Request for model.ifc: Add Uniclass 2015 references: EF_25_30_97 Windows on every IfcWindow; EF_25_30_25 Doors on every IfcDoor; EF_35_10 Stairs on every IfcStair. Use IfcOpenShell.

First a look at what the model holds.

```python
import ifcopenshell

model = ifcopenshell.open("model.ifc")
print(model.schema)
print("classifications:", [c.Name for c in model.by_type("IfcClassification")])
for ifc_class in ("IfcDoor", "IfcRoof", "IfcStair", "IfcWall", "IfcWindow"):
    print(ifc_class, len(model.by_type(ifc_class)))
```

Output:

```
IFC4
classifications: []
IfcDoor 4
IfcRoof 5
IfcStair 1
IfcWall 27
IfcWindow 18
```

```python
import ifcopenshell
import ifcopenshell.api.classification

model = ifcopenshell.open("model.ifc")

system = ifcopenshell.api.classification.add_classification(model, classification="Uniclass 2015")

codes = {
    "IfcWindow": ("EF_25_30_97", "Windows"),
    "IfcDoor": ("EF_25_30_25", "Doors"),
    "IfcStair": ("EF_35_10", "Stairs"),
}
for ifc_class, (code, name) in codes.items():
    products = model.by_type(ifc_class)
    ifcopenshell.api.classification.add_reference(
        model, products=products, classification=system, identification=code, name=name
    )
    print(code, len(products))

model.write("model_rev.ifc")
```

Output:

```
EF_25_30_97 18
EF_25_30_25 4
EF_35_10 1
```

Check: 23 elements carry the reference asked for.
